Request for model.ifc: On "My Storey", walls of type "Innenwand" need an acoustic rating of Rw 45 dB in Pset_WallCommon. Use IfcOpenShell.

First a look at what the model holds.

```python
import ifcopenshell
import ifcopenshell.util.element

model = ifcopenshell.open("model.ifc")
print(model.schema)
storey = next(s for s in model.by_type("IfcBuildingStorey") if s.Name == "My Storey")
walls = [e for e in ifcopenshell.util.element.get_decomposition(storey) if e.is_a("IfcWall")]
seen = {}
for e in walls:
    element_type = ifcopenshell.util.element.get_type(e)
    key = (element_type.Name if element_type != e and element_type else None, ifcopenshell.util.element.get_pset(e, "Pset_WallCommon", "AcousticRating"))
    seen[key] = seen.get(key, 0) + 1
for (name, value), count in sorted(seen.items(), key=str):
    print(count, "x", name, "|", value)
```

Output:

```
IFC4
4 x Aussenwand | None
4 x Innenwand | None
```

```python
import ifcopenshell
import ifcopenshell.api.pset
import ifcopenshell.util.element

model = ifcopenshell.open("model.ifc")

storey = next(s for s in model.by_type("IfcBuildingStorey") if s.Name == "My Storey")
walls = [e for e in ifcopenshell.util.element.get_decomposition(storey) if e.is_a("IfcWall")]

count = 0
for e in walls:
    element_type = ifcopenshell.util.element.get_type(e)
    if element_type in (None, e) or element_type.Name != "Innenwand":
        continue
    # add_pset returns the element's existing set when there is one.
    pset = ifcopenshell.api.pset.add_pset(model, product=e, name="Pset_WallCommon")
    ifcopenshell.api.pset.edit_pset(model, pset=pset, properties={"AcousticRating": "Rw 45 dB"})
    count += 1

print(count, "walls updated")

model.write("model_rev.ifc")
```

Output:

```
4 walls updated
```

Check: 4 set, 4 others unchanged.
